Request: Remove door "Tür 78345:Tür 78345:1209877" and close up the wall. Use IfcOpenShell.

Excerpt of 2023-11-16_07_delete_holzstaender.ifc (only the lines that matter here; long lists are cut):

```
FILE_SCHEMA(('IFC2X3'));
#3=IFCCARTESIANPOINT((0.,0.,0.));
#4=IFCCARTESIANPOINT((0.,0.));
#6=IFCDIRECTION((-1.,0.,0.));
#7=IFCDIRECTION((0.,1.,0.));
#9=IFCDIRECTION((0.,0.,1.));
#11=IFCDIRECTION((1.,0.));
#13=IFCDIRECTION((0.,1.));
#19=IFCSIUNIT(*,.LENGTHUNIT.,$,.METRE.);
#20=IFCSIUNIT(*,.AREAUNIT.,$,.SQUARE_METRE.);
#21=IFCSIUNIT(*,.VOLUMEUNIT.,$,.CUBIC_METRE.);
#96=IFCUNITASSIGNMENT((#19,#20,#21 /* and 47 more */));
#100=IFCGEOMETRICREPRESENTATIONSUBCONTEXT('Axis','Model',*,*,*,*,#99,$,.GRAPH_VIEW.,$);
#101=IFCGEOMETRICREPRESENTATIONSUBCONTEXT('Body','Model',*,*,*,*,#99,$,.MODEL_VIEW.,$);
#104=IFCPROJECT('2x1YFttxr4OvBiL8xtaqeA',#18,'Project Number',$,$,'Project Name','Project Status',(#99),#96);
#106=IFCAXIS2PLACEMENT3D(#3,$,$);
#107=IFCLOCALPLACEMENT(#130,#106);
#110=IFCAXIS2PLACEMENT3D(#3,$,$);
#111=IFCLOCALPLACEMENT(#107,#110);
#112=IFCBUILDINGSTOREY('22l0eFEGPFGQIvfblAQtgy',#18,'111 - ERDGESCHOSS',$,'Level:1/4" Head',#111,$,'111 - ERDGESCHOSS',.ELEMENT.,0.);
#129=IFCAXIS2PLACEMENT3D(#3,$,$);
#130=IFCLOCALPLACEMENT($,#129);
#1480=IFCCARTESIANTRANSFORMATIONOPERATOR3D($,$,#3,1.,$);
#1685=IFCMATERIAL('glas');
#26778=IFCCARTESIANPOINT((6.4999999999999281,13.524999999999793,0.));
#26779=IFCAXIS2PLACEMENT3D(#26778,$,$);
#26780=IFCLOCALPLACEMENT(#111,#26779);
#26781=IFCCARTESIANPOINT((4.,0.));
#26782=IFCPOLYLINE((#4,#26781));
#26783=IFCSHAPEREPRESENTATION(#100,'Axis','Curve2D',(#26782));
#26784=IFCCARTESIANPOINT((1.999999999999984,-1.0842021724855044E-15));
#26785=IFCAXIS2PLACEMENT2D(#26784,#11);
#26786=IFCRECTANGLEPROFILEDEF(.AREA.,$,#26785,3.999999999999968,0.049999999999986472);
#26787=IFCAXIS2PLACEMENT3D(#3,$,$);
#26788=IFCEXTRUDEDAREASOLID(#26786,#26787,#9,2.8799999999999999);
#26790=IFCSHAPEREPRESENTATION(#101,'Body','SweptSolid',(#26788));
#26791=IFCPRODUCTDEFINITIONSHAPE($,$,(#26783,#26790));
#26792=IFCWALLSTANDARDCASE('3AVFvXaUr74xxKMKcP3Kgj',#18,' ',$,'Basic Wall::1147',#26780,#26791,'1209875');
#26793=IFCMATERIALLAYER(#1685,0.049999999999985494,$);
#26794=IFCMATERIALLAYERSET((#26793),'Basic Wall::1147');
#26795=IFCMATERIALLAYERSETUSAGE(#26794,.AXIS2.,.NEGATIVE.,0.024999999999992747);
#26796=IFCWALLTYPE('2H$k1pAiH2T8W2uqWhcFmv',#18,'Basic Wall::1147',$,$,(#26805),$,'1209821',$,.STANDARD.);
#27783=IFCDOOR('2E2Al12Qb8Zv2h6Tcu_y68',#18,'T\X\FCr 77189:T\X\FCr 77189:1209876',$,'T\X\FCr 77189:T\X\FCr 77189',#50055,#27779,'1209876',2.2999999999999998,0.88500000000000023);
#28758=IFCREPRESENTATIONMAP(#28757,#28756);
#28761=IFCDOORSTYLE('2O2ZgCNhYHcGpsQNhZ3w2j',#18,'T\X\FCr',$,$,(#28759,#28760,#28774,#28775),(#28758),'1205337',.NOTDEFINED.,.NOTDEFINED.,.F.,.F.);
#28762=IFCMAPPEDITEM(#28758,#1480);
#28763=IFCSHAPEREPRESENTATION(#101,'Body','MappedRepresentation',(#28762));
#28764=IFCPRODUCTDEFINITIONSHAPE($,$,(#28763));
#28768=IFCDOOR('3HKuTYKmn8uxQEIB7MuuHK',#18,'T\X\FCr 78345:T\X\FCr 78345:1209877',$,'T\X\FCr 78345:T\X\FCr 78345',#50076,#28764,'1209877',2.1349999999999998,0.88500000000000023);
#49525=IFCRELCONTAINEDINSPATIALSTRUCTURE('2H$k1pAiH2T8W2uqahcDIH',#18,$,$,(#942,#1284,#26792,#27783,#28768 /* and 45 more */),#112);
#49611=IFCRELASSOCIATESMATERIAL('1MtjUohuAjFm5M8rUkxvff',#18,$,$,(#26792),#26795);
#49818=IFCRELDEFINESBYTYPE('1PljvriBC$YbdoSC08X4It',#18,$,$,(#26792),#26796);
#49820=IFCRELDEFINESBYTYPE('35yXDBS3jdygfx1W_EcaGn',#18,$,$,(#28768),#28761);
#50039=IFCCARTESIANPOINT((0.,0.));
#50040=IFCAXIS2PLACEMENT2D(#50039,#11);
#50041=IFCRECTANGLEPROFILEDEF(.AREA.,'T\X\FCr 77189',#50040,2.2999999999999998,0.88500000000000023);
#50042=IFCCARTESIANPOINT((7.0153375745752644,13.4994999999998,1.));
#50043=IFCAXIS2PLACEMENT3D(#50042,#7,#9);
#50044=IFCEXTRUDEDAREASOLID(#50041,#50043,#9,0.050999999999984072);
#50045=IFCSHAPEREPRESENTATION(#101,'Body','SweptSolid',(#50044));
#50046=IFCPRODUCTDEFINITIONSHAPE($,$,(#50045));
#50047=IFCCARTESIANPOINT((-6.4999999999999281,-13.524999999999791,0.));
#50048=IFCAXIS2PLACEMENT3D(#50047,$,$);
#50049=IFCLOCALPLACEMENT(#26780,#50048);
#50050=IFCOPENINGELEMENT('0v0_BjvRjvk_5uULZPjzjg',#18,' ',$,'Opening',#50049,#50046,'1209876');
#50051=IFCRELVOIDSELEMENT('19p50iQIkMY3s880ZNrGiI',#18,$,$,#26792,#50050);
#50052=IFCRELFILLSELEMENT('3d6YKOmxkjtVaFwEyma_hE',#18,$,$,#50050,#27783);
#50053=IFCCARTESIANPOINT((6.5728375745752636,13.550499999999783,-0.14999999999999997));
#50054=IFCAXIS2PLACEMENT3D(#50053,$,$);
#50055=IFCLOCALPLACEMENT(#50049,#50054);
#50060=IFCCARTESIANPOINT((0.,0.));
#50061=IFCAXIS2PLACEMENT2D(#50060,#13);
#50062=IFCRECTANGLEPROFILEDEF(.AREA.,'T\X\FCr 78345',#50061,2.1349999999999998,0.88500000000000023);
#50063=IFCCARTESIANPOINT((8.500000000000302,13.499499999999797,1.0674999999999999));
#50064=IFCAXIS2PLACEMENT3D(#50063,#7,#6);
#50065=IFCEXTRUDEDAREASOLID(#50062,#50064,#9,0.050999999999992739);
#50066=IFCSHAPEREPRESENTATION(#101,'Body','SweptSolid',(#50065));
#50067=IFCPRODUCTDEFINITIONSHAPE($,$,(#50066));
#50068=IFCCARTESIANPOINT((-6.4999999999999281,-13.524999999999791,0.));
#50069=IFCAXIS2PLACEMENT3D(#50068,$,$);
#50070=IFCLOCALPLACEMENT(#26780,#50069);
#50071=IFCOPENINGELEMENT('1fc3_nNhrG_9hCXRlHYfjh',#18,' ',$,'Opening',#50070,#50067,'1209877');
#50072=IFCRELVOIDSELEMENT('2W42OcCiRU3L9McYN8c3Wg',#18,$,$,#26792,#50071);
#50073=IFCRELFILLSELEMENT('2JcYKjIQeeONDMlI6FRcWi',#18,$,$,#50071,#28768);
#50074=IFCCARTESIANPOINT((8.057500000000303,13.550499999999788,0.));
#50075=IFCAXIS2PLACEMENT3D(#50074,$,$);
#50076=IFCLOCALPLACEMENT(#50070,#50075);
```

```python
import ifcopenshell
import ifcopenshell.api.feature
import ifcopenshell.api.root
import ifcopenshell.geom
import ifcopenshell.util.shape

model = ifcopenshell.open("2023-11-16_07_delete_holzstaender.ifc")
settings = ifcopenshell.geom.settings()


def volume(element):
    """Net volume in cubic metres, openings subtracted."""
    shape = ifcopenshell.geom.create_shape(settings, element)
    return ifcopenshell.util.shape.get_volume(shape.geometry)


door = model.by_guid("3HKuTYKmn8uxQEIB7MuuHK")
opening = door.FillsVoids[0].RelatingOpeningElement
wall = opening.VoidsElements[0].RelatingBuildingElement
before = volume(wall)

ifcopenshell.api.root.remove_product(model, product=door)
ifcopenshell.api.feature.remove_feature(model, feature=opening)

after = volume(wall)

print(f"wall volume {before:.3f} -> {after:.3f} m3")

model.write("2023-11-16_07_delete_holzstaender-out.ifc")
```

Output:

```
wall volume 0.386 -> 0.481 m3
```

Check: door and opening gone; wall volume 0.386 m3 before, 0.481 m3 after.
